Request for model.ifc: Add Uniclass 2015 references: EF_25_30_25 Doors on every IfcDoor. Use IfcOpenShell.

First a look at what the model holds.

```python
import ifcopenshell

model = ifcopenshell.open("model.ifc")
print(model.schema)
print("classifications:", [c.Name for c in model.by_type("IfcClassification")])
for ifc_class in ("IfcDoor", "IfcRoof", "IfcStair", "IfcWall", "IfcWindow"):
    print(ifc_class, len(model.by_type(ifc_class)))
```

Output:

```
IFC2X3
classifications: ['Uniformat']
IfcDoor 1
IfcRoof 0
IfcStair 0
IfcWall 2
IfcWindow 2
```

```python
import ifcopenshell
import ifcopenshell.api.classification

model = ifcopenshell.open("model.ifc")

# IFC2X3 requires Source and Edition and has no link from the project to the system.
system = model.create_entity("IfcClassification", Source="NBS", Edition="2015", Name="Uniclass 2015")

codes = {
    "IfcDoor": ("EF_25_30_25", "Doors"),
}
for ifc_class, (code, name) in codes.items():
    products = model.by_type(ifc_class)
    ifcopenshell.api.classification.add_reference(
        model, products=products, classification=system, identification=code, name=name
    )
    print(code, len(products))

model.write("model_v2.ifc")
```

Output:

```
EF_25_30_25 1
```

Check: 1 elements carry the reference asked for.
